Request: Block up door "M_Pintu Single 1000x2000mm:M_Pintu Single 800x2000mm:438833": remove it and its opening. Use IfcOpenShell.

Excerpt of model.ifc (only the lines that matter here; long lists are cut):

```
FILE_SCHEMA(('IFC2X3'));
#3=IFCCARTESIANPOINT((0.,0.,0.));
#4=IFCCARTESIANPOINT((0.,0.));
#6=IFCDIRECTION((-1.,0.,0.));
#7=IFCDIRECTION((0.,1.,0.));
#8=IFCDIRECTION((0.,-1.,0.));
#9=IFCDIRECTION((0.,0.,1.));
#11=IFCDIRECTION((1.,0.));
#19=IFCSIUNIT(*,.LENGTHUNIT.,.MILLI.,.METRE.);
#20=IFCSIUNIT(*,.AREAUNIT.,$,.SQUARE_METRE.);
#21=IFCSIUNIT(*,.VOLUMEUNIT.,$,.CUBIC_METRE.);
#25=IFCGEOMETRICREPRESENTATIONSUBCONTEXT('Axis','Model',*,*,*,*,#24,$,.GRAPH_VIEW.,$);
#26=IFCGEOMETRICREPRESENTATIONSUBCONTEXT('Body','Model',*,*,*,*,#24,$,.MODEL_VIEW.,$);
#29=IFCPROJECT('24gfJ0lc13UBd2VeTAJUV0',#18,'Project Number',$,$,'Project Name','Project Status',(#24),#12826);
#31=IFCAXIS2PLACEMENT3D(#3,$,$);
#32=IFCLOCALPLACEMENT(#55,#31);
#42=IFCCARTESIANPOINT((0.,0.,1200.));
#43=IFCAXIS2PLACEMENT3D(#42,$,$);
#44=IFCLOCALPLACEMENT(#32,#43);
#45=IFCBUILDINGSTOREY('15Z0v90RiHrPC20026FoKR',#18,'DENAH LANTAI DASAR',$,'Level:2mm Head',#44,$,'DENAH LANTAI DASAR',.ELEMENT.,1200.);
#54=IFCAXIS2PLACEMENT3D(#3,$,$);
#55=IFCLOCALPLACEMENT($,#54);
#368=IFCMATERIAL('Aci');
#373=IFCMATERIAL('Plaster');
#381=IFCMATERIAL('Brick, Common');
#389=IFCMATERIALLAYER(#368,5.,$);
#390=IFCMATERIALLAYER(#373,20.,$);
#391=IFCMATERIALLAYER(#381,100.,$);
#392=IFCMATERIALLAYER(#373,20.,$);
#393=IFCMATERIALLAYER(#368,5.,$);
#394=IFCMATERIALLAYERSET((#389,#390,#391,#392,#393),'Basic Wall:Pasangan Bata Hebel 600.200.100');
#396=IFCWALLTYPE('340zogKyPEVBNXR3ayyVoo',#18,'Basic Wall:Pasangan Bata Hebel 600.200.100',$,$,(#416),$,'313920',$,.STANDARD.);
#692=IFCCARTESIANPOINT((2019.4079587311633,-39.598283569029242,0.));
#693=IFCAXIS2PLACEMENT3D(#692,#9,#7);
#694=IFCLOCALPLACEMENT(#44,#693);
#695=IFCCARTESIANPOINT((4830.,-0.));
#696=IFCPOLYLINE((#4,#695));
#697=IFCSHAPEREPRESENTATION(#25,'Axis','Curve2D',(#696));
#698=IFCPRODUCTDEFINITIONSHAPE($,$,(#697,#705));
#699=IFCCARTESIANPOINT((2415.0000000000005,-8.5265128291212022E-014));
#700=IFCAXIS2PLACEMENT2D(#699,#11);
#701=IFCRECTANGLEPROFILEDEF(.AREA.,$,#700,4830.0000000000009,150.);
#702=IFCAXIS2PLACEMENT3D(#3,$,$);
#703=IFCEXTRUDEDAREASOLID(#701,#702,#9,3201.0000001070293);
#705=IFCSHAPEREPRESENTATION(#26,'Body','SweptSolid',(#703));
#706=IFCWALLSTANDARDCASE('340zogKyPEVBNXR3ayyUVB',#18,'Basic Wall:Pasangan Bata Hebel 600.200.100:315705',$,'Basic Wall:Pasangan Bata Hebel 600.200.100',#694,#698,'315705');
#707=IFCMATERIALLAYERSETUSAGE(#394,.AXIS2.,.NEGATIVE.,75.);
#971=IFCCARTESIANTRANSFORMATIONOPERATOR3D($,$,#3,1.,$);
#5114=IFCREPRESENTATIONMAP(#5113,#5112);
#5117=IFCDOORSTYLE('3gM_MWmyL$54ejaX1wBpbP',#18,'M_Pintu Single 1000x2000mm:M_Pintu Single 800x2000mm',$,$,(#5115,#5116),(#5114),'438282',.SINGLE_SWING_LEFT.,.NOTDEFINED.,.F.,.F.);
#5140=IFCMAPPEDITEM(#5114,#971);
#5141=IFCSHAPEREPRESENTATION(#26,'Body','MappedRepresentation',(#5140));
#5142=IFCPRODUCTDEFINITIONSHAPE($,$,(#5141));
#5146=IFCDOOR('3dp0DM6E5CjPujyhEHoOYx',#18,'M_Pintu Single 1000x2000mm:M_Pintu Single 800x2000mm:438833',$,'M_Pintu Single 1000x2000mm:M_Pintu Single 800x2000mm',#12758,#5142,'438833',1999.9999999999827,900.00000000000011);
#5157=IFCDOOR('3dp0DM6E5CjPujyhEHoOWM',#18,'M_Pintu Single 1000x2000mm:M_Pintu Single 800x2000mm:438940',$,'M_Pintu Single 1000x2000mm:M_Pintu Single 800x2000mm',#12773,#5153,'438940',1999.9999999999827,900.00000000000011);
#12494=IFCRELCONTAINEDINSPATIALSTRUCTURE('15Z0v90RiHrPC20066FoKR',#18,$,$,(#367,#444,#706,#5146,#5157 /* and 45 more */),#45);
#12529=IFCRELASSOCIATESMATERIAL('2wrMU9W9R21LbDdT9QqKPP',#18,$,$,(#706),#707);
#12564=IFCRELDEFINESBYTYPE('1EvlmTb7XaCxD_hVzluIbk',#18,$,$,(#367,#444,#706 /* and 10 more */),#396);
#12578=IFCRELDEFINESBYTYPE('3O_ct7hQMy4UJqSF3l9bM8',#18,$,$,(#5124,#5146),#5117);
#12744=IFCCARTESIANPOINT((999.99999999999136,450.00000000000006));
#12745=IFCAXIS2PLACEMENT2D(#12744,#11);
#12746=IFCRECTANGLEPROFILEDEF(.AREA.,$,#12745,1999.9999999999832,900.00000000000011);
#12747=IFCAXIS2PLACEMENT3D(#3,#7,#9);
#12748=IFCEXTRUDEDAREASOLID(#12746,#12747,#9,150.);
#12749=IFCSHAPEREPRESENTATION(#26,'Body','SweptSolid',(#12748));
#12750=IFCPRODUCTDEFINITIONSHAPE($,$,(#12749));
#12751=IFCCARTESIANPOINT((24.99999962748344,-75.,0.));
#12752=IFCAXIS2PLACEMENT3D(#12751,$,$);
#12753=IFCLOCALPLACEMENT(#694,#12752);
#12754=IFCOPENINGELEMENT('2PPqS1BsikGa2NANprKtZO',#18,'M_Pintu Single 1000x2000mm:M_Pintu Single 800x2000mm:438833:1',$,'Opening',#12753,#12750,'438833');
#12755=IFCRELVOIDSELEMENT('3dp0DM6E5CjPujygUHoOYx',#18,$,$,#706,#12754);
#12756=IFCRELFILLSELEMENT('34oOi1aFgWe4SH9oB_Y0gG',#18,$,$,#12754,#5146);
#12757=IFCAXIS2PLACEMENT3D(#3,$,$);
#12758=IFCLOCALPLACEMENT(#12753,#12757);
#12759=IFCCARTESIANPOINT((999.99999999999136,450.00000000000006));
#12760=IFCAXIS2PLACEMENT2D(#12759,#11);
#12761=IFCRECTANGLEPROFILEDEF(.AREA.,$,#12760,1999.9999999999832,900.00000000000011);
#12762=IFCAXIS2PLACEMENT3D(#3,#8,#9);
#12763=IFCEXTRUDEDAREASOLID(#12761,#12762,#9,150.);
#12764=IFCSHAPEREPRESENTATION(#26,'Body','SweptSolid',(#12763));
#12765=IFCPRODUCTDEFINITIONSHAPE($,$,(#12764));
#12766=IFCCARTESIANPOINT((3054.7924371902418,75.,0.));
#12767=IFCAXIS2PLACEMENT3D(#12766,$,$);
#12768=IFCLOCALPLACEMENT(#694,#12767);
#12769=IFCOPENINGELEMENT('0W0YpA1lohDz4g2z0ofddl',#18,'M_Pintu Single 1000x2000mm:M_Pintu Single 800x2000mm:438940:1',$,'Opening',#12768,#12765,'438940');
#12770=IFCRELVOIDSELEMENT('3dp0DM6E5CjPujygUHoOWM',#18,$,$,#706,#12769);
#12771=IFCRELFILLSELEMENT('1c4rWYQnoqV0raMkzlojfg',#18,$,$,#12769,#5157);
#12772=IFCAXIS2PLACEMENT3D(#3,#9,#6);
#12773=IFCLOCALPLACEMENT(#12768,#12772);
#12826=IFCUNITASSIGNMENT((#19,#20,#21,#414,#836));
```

```python
import ifcopenshell
import ifcopenshell.api.feature
import ifcopenshell.api.root
import ifcopenshell.geom
import ifcopenshell.util.shape

model = ifcopenshell.open("model.ifc")
settings = ifcopenshell.geom.settings()


def volume(element):
    """Net volume in cubic metres, openings subtracted."""
    shape = ifcopenshell.geom.create_shape(settings, element)
    return ifcopenshell.util.shape.get_volume(shape.geometry)


door = model.by_guid("3dp0DM6E5CjPujyhEHoOYx")
opening = door.FillsVoids[0].RelatingOpeningElement
wall = opening.VoidsElements[0].RelatingBuildingElement
before = volume(wall)

ifcopenshell.api.root.remove_product(model, product=door)
ifcopenshell.api.feature.remove_feature(model, feature=opening)

after = volume(wall)

print(f"wall volume {before:.3f} -> {after:.3f} m3")

model.write("model_v2.ifc")
```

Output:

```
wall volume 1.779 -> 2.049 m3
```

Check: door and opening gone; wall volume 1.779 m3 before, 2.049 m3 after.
